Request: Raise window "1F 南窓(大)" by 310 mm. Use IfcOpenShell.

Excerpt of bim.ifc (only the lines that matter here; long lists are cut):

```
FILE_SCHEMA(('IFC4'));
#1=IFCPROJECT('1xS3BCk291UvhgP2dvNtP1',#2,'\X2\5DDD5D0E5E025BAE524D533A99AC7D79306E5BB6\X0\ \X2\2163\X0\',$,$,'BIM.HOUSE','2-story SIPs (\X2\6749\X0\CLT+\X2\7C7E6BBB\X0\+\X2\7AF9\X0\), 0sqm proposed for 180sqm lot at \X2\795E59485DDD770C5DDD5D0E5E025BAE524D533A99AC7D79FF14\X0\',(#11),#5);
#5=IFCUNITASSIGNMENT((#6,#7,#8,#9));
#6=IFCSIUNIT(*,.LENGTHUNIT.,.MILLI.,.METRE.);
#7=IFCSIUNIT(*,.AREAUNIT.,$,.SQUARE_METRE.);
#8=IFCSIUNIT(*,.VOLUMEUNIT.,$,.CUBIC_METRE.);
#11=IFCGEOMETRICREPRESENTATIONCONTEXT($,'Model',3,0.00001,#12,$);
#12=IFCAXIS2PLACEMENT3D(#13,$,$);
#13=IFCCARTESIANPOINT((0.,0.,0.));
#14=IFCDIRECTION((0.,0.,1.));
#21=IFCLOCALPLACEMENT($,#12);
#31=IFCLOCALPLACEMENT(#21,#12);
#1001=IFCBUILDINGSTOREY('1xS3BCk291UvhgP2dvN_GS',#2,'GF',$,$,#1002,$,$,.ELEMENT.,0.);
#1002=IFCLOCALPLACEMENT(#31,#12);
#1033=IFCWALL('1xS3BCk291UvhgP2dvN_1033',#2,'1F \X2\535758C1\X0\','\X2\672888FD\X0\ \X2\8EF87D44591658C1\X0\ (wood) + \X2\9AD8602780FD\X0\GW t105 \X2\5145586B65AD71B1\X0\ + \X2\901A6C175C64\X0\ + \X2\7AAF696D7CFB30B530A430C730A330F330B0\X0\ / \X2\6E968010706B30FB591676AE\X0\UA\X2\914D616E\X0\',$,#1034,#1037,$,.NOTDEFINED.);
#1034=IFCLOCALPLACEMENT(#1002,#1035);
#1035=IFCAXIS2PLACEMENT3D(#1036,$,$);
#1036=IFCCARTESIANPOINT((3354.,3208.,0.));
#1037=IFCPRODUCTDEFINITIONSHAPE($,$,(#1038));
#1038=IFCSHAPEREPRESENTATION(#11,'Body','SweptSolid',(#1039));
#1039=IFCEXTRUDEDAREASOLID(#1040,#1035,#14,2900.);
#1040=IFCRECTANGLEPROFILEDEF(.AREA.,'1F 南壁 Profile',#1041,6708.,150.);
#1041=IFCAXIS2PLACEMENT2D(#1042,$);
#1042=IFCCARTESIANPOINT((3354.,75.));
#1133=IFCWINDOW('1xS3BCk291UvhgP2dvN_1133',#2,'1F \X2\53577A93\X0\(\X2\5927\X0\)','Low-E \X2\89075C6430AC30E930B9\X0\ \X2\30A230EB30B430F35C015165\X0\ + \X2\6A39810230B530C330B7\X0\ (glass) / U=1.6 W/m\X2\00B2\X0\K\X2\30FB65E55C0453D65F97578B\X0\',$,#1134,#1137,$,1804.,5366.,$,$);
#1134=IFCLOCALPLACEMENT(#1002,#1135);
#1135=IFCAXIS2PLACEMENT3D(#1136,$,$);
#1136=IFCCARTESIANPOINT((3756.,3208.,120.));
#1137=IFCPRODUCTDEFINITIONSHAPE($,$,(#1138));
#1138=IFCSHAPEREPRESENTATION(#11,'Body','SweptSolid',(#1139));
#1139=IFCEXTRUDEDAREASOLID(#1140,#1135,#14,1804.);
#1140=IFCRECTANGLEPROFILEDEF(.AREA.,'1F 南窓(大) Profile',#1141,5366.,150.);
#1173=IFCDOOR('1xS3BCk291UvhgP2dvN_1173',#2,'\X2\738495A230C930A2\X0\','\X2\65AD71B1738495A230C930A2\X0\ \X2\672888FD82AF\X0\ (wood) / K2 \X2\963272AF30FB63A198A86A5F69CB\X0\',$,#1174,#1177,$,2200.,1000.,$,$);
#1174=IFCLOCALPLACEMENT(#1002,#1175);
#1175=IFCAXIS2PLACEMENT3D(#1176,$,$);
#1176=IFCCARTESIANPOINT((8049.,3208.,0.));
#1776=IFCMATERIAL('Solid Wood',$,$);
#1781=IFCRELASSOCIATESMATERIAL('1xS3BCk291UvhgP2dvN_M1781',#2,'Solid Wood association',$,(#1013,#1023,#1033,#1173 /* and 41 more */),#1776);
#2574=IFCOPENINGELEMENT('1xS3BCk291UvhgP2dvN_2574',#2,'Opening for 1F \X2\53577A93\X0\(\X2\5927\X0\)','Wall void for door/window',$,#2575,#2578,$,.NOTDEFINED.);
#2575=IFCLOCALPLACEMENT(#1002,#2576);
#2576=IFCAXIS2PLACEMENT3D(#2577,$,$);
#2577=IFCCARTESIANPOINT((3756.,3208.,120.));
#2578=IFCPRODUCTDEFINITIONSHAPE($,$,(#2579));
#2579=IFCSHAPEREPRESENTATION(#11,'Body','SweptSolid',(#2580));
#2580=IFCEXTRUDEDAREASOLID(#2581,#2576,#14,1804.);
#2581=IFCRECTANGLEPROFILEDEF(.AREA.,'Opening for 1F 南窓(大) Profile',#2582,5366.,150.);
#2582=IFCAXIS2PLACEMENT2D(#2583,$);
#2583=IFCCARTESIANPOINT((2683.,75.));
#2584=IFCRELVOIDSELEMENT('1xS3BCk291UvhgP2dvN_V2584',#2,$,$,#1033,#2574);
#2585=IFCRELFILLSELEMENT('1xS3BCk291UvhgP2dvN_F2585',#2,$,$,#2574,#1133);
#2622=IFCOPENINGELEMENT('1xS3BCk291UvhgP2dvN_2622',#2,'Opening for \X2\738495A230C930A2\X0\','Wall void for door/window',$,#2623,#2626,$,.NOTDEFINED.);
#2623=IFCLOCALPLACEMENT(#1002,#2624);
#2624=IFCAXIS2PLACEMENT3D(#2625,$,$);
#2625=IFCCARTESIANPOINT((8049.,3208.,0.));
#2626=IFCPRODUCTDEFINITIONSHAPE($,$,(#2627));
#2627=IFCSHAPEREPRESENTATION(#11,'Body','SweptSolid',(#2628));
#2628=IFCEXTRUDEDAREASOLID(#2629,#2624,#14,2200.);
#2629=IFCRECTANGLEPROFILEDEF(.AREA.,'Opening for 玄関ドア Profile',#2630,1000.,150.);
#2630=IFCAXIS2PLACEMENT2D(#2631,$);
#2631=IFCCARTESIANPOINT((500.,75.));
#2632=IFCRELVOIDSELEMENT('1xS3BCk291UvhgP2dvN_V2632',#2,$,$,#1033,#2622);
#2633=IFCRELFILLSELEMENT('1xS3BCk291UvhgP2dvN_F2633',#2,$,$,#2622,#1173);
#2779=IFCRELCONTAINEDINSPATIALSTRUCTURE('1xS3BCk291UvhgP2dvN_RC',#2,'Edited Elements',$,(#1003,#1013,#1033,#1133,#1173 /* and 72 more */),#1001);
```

```python
import numpy as np
import ifcopenshell
import ifcopenshell.api.geometry
import ifcopenshell.util.placement
import ifcopenshell.util.unit

model = ifcopenshell.open("bim.ifc")
unit_scale = ifcopenshell.util.unit.calculate_unit_scale(model)

window = model.by_guid("1xS3BCk291UvhgP2dvN_1133")
opening = window.FillsVoids[0].RelatingOpeningElement
dz = 0.31 / unit_scale

shift = np.array([0.0, 0.0, dz])
# The window is not placed relative to its opening, so move both.
for product in (opening, window):
    matrix = ifcopenshell.util.placement.get_local_placement(product.ObjectPlacement)
    matrix[:3, 3] += shift
    ifcopenshell.api.geometry.edit_object_placement(model, product=product, matrix=matrix, is_si=False)

print(f"moved by {dz * unit_scale:+.3f} m")

model.write("bim-out.ifc")
```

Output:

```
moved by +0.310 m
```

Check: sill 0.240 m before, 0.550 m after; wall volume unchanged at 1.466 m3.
